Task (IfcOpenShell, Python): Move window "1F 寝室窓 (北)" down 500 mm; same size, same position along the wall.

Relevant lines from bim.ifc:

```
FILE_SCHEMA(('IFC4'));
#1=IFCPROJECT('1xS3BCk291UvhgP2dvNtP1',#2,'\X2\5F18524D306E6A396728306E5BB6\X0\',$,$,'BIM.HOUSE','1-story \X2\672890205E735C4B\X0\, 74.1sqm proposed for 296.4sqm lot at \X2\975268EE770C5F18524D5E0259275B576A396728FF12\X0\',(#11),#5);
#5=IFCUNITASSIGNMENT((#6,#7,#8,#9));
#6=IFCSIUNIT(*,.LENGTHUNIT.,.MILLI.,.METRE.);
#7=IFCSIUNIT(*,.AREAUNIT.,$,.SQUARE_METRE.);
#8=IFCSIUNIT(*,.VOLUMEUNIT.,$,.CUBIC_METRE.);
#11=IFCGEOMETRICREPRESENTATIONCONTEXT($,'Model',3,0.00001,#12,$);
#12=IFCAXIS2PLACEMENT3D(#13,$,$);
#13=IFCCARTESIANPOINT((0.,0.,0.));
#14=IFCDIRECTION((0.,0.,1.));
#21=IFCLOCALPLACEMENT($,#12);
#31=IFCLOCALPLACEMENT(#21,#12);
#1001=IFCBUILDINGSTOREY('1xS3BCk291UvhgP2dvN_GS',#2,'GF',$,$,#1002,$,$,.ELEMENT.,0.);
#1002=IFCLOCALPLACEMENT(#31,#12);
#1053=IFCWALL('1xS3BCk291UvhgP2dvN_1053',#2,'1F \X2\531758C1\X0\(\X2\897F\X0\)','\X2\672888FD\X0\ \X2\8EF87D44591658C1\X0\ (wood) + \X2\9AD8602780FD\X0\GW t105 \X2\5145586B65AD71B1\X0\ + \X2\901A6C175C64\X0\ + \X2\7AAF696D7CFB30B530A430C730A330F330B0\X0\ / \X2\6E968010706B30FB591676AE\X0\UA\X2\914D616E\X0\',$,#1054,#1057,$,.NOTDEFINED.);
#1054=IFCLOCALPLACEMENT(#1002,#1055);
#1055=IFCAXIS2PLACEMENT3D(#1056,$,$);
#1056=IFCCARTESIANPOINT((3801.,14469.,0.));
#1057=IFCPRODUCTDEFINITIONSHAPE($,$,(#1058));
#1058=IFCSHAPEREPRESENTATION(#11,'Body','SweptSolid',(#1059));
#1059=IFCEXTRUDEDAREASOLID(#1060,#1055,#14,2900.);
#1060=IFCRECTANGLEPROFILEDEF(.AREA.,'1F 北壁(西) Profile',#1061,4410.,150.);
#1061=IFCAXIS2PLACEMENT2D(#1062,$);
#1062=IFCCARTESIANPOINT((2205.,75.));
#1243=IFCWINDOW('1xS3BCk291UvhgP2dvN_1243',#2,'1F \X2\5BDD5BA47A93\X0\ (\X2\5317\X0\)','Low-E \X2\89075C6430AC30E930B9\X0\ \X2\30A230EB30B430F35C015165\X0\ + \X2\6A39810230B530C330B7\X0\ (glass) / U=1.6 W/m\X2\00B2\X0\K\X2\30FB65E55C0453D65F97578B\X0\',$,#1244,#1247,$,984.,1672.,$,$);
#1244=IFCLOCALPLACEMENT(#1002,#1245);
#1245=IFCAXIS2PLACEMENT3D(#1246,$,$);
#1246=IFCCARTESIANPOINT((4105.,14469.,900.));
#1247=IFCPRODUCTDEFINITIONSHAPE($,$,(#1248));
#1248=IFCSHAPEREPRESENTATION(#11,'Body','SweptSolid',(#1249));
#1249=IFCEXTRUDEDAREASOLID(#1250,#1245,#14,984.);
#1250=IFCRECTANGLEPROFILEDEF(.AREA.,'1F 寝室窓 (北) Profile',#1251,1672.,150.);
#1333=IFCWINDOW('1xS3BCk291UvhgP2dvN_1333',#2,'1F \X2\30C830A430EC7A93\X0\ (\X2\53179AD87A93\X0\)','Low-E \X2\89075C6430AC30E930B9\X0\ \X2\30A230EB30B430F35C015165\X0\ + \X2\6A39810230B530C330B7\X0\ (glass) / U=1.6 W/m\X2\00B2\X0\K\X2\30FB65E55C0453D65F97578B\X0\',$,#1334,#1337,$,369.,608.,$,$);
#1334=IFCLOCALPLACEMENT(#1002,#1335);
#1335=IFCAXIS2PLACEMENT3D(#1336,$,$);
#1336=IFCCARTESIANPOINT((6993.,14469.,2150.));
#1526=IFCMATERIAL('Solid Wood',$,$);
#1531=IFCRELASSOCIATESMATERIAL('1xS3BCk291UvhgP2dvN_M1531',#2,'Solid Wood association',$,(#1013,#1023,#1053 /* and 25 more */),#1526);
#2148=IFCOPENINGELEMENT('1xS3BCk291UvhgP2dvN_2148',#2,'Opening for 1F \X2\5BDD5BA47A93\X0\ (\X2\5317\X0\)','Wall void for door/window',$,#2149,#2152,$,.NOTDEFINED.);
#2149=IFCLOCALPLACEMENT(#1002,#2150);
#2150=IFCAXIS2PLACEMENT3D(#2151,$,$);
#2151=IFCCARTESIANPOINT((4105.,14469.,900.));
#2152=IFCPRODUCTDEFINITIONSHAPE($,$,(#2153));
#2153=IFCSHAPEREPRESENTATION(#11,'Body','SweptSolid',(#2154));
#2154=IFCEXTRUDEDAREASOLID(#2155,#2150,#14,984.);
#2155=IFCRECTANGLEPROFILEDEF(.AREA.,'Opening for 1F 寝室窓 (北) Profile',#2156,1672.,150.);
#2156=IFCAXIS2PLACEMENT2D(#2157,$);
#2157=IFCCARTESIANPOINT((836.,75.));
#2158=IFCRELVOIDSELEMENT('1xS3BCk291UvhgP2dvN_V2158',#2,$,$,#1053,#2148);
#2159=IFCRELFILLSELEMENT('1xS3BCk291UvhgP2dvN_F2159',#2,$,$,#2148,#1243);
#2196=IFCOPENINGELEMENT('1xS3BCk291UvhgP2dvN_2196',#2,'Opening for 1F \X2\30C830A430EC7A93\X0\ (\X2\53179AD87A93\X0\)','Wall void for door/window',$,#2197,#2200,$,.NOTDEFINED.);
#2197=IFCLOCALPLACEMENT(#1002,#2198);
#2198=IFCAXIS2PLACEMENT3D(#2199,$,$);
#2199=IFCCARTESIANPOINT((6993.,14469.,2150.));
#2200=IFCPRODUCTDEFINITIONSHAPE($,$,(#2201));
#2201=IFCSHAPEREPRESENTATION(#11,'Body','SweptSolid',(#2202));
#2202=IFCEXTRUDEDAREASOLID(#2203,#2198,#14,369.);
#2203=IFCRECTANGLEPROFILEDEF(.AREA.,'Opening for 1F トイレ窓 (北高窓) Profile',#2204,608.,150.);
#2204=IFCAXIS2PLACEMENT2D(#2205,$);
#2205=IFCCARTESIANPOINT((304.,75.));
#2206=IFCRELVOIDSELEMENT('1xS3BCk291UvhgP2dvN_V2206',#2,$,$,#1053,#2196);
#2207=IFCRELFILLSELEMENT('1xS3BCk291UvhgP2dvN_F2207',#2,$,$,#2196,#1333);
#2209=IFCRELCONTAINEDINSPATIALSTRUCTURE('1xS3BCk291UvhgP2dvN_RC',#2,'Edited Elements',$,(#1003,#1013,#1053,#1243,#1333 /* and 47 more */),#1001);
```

```python
import numpy as np
import ifcopenshell
import ifcopenshell.api.geometry
import ifcopenshell.util.placement
import ifcopenshell.util.unit

model = ifcopenshell.open("bim.ifc")
unit_scale = ifcopenshell.util.unit.calculate_unit_scale(model)

window = model.by_id(1243)
opening = window.FillsVoids[0].RelatingOpeningElement
dz = -500.0

shift = np.array([0.0, 0.0, dz])
# The window is not placed relative to its opening, so move both.
for product in (opening, window):
    matrix = ifcopenshell.util.placement.get_local_placement(product.ObjectPlacement)
    matrix[:3, 3] += shift
    ifcopenshell.api.geometry.edit_object_placement(model, product=product, matrix=matrix, is_si=False)

print(f"moved by {dz * unit_scale:+.3f} m")

model.write("bim_v2.ifc")
```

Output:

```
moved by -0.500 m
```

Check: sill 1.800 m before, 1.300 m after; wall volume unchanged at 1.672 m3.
